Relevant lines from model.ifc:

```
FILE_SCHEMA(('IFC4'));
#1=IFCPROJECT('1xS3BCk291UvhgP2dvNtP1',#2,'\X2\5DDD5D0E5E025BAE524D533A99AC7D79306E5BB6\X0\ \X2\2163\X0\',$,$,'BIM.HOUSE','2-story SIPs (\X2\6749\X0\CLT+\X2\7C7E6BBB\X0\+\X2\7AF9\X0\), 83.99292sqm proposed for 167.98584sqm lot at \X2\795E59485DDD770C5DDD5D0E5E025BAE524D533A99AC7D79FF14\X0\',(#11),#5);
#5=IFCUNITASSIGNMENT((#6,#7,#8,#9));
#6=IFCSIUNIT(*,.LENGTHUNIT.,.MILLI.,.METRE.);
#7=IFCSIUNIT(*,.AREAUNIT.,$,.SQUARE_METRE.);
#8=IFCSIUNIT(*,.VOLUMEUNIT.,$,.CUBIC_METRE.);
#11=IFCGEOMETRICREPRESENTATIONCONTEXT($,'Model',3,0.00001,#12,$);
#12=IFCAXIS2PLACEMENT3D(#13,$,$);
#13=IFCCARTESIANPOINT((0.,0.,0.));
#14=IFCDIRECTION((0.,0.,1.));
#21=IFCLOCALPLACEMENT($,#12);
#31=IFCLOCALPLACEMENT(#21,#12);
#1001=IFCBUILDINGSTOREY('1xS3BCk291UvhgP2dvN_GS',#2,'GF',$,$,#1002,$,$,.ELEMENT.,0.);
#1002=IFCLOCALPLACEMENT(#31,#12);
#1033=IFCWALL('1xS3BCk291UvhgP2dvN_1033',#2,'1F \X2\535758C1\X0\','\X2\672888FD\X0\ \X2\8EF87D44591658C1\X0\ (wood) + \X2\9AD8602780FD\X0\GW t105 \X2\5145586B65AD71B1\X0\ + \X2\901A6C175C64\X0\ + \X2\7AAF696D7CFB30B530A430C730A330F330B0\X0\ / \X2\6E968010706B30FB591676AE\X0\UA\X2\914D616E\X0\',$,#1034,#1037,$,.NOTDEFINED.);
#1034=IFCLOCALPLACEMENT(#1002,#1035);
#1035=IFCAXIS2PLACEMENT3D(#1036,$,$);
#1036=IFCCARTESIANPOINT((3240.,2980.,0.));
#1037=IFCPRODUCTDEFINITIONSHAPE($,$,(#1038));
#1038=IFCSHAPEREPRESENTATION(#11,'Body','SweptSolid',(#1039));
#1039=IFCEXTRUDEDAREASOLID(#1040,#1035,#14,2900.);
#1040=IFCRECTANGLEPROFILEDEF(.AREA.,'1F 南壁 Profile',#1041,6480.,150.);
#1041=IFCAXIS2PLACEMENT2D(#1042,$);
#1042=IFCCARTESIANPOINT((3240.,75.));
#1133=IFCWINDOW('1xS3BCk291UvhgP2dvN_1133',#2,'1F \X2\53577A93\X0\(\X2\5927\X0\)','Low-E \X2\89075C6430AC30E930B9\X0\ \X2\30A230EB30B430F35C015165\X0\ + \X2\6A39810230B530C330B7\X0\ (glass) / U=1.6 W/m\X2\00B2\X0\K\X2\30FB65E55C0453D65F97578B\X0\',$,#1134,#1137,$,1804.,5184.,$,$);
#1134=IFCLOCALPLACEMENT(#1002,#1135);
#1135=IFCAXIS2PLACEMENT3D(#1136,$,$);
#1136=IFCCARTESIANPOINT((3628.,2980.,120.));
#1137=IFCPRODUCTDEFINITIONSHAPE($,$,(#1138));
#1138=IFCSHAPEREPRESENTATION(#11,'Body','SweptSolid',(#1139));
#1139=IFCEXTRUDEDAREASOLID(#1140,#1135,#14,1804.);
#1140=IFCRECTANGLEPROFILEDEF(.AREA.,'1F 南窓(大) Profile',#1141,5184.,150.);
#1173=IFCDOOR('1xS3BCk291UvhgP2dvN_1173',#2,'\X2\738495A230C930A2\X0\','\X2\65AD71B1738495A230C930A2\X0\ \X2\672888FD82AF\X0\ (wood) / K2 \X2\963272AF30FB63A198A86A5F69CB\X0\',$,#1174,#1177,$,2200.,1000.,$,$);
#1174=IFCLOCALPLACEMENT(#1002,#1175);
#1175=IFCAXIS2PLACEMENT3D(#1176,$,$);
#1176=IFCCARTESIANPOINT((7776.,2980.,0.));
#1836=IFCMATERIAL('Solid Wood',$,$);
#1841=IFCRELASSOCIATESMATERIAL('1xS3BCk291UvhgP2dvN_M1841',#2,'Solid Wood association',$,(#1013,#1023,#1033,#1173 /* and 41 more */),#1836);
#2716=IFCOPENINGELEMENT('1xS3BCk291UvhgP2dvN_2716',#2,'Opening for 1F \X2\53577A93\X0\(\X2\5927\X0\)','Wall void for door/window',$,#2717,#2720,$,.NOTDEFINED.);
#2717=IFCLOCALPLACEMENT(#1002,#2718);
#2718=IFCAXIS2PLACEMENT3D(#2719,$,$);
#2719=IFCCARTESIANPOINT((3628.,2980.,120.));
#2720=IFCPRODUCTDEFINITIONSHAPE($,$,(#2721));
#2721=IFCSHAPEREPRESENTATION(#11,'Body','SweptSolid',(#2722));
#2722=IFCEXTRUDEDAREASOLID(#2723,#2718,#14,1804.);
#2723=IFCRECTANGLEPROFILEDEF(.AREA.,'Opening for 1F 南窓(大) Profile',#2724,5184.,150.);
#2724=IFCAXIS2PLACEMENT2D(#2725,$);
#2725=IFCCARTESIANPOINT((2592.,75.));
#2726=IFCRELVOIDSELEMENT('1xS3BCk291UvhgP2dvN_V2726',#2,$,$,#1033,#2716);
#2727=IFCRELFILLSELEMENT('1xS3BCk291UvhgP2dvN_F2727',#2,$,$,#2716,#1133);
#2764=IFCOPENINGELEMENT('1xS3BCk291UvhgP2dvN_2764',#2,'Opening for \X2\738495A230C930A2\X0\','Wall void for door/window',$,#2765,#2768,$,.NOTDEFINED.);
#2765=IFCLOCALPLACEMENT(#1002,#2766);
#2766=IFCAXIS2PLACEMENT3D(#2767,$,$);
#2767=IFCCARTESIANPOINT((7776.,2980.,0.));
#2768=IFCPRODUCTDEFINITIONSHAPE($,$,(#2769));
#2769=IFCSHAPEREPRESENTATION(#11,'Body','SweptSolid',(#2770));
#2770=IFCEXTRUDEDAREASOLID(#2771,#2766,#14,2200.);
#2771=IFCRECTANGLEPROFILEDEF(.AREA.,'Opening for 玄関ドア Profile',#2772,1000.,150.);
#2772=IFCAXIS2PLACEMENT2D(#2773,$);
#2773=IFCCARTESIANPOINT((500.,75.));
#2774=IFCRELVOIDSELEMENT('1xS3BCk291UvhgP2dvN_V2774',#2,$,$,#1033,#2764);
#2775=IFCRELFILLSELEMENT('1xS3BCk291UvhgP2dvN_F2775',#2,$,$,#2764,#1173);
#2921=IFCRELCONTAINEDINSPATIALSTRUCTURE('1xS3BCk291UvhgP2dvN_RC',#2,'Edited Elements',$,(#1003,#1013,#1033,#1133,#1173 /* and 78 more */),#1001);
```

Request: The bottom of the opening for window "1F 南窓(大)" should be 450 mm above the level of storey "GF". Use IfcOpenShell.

```python
import numpy as np
import ifcopenshell
import ifcopenshell.api.geometry
import ifcopenshell.geom
import ifcopenshell.util.element
import ifcopenshell.util.placement
import ifcopenshell.util.shape
import ifcopenshell.util.unit

model = ifcopenshell.open("model.ifc")
unit_scale = ifcopenshell.util.unit.calculate_unit_scale(model)

window = model.by_guid("1xS3BCk291UvhgP2dvN_1133")
opening = window.FillsVoids[0].RelatingOpeningElement
storey = ifcopenshell.util.element.get_container(window, ifc_class="IfcBuildingStorey")
level = ifcopenshell.util.placement.get_local_placement(storey.ObjectPlacement)[2, 3]

# The opening's origin need not be at the sill, so measure its lowest point.
shape = ifcopenshell.geom.create_shape(ifcopenshell.geom.settings(), opening)
bottom = ifcopenshell.util.shape.get_shape_bottom_elevation(shape, shape.geometry) / unit_scale
dz = level + 0.45 / unit_scale - bottom

shift = np.array([0.0, 0.0, dz])
# The window is not placed relative to its opening, so move both.
for product in (opening, window):
    matrix = ifcopenshell.util.placement.get_local_placement(product.ObjectPlacement)
    matrix[:3, 3] += shift
    ifcopenshell.api.geometry.edit_object_placement(model, product=product, matrix=matrix, is_si=False)

print(f"moved by {dz * unit_scale:+.3f} m")

model.write("model_v2.ifc")
```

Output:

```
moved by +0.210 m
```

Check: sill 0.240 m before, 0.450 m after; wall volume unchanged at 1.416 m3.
